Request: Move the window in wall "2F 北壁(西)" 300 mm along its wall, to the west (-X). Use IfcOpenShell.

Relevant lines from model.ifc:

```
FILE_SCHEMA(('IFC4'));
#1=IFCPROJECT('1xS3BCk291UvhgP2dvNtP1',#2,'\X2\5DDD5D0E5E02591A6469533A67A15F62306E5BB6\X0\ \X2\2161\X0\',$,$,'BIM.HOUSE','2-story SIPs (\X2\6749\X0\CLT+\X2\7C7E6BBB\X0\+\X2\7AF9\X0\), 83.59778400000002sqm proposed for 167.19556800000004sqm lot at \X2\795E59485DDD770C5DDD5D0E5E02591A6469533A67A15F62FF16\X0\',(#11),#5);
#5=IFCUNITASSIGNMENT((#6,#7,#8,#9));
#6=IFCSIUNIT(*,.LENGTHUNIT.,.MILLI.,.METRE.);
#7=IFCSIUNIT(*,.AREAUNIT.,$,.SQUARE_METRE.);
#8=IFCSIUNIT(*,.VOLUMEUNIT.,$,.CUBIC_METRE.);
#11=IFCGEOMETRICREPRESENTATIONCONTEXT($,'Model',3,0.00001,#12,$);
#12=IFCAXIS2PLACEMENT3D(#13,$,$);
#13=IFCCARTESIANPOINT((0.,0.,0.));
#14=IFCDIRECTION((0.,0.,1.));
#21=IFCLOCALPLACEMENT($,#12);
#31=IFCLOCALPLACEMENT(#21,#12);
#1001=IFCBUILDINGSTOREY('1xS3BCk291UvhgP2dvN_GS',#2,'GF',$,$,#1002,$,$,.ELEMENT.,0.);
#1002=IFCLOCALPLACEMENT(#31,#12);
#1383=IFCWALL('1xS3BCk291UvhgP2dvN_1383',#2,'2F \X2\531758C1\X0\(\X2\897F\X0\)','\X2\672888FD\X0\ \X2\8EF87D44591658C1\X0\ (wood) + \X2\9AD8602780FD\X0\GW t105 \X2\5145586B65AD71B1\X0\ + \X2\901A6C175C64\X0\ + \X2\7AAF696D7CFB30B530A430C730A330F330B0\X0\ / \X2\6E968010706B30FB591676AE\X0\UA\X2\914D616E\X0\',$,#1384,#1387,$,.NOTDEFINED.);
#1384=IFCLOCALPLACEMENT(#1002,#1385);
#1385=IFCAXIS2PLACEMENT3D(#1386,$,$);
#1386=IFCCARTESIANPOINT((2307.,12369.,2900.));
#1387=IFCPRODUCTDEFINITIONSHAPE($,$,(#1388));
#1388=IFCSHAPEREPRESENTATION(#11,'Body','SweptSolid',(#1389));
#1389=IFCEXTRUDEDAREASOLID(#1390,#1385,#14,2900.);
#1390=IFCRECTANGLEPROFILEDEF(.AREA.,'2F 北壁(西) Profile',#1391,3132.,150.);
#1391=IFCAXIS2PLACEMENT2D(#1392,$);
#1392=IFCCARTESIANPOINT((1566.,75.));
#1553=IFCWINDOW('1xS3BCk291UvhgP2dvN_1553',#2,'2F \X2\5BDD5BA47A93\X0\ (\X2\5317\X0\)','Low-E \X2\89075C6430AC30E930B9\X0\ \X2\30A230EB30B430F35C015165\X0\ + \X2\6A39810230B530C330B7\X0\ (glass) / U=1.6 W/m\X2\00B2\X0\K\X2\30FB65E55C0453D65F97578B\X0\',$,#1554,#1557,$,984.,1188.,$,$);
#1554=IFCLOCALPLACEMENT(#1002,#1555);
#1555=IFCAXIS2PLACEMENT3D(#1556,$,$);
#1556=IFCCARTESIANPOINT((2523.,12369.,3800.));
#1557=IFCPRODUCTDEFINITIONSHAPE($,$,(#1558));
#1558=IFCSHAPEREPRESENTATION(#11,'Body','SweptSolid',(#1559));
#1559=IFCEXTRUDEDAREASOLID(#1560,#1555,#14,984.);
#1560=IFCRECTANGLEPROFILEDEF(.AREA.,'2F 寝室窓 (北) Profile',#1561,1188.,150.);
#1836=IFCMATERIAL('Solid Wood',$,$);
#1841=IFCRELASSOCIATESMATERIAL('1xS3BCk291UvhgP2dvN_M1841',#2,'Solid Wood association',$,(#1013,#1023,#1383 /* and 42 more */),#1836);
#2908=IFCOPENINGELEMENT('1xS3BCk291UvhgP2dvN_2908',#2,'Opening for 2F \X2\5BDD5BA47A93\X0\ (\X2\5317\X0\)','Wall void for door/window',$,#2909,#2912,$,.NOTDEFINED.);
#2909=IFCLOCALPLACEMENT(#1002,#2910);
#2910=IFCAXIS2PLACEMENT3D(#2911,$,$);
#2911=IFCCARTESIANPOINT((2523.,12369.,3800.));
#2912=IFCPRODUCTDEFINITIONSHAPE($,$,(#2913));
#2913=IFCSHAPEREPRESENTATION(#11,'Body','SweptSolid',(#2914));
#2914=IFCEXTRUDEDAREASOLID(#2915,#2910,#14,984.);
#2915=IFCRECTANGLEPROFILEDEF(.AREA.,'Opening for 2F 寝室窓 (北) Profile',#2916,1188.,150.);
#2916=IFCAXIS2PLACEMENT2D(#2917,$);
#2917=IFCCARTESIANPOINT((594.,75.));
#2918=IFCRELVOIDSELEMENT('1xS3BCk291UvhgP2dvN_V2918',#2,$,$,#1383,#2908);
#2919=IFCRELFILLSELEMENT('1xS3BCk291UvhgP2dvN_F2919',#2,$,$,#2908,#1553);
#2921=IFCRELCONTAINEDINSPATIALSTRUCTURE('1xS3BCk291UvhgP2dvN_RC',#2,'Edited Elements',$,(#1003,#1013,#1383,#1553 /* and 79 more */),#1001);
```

```python
import ifcopenshell
import ifcopenshell.api.geometry
import ifcopenshell.util.placement

model = ifcopenshell.open("model.ifc")

window = model.by_guid("1xS3BCk291UvhgP2dvN_1553")
opening = window.FillsVoids[0].RelatingOpeningElement
wall = opening.VoidsElements[0].RelatingBuildingElement

wall_matrix = ifcopenshell.util.placement.get_local_placement(wall.ObjectPlacement)
shift = wall_matrix[:3, 0] * -300.0
before = ifcopenshell.util.placement.get_local_placement(window.ObjectPlacement)[:3, 3].copy()

# The window is not placed relative to its opening, so move both.
for product in (opening, window):
    matrix = ifcopenshell.util.placement.get_local_placement(product.ObjectPlacement)
    matrix[:3, 3] += shift
    ifcopenshell.api.geometry.edit_object_placement(model, product=product, matrix=matrix, is_si=False)

after = ifcopenshell.util.placement.get_local_placement(window.ObjectPlacement)[:3, 3]
print("window moved by", (after - before).round(3) + 0.0)

model.write("model_v2.ifc")
```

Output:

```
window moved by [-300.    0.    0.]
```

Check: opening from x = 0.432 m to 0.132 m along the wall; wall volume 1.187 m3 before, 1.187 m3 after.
